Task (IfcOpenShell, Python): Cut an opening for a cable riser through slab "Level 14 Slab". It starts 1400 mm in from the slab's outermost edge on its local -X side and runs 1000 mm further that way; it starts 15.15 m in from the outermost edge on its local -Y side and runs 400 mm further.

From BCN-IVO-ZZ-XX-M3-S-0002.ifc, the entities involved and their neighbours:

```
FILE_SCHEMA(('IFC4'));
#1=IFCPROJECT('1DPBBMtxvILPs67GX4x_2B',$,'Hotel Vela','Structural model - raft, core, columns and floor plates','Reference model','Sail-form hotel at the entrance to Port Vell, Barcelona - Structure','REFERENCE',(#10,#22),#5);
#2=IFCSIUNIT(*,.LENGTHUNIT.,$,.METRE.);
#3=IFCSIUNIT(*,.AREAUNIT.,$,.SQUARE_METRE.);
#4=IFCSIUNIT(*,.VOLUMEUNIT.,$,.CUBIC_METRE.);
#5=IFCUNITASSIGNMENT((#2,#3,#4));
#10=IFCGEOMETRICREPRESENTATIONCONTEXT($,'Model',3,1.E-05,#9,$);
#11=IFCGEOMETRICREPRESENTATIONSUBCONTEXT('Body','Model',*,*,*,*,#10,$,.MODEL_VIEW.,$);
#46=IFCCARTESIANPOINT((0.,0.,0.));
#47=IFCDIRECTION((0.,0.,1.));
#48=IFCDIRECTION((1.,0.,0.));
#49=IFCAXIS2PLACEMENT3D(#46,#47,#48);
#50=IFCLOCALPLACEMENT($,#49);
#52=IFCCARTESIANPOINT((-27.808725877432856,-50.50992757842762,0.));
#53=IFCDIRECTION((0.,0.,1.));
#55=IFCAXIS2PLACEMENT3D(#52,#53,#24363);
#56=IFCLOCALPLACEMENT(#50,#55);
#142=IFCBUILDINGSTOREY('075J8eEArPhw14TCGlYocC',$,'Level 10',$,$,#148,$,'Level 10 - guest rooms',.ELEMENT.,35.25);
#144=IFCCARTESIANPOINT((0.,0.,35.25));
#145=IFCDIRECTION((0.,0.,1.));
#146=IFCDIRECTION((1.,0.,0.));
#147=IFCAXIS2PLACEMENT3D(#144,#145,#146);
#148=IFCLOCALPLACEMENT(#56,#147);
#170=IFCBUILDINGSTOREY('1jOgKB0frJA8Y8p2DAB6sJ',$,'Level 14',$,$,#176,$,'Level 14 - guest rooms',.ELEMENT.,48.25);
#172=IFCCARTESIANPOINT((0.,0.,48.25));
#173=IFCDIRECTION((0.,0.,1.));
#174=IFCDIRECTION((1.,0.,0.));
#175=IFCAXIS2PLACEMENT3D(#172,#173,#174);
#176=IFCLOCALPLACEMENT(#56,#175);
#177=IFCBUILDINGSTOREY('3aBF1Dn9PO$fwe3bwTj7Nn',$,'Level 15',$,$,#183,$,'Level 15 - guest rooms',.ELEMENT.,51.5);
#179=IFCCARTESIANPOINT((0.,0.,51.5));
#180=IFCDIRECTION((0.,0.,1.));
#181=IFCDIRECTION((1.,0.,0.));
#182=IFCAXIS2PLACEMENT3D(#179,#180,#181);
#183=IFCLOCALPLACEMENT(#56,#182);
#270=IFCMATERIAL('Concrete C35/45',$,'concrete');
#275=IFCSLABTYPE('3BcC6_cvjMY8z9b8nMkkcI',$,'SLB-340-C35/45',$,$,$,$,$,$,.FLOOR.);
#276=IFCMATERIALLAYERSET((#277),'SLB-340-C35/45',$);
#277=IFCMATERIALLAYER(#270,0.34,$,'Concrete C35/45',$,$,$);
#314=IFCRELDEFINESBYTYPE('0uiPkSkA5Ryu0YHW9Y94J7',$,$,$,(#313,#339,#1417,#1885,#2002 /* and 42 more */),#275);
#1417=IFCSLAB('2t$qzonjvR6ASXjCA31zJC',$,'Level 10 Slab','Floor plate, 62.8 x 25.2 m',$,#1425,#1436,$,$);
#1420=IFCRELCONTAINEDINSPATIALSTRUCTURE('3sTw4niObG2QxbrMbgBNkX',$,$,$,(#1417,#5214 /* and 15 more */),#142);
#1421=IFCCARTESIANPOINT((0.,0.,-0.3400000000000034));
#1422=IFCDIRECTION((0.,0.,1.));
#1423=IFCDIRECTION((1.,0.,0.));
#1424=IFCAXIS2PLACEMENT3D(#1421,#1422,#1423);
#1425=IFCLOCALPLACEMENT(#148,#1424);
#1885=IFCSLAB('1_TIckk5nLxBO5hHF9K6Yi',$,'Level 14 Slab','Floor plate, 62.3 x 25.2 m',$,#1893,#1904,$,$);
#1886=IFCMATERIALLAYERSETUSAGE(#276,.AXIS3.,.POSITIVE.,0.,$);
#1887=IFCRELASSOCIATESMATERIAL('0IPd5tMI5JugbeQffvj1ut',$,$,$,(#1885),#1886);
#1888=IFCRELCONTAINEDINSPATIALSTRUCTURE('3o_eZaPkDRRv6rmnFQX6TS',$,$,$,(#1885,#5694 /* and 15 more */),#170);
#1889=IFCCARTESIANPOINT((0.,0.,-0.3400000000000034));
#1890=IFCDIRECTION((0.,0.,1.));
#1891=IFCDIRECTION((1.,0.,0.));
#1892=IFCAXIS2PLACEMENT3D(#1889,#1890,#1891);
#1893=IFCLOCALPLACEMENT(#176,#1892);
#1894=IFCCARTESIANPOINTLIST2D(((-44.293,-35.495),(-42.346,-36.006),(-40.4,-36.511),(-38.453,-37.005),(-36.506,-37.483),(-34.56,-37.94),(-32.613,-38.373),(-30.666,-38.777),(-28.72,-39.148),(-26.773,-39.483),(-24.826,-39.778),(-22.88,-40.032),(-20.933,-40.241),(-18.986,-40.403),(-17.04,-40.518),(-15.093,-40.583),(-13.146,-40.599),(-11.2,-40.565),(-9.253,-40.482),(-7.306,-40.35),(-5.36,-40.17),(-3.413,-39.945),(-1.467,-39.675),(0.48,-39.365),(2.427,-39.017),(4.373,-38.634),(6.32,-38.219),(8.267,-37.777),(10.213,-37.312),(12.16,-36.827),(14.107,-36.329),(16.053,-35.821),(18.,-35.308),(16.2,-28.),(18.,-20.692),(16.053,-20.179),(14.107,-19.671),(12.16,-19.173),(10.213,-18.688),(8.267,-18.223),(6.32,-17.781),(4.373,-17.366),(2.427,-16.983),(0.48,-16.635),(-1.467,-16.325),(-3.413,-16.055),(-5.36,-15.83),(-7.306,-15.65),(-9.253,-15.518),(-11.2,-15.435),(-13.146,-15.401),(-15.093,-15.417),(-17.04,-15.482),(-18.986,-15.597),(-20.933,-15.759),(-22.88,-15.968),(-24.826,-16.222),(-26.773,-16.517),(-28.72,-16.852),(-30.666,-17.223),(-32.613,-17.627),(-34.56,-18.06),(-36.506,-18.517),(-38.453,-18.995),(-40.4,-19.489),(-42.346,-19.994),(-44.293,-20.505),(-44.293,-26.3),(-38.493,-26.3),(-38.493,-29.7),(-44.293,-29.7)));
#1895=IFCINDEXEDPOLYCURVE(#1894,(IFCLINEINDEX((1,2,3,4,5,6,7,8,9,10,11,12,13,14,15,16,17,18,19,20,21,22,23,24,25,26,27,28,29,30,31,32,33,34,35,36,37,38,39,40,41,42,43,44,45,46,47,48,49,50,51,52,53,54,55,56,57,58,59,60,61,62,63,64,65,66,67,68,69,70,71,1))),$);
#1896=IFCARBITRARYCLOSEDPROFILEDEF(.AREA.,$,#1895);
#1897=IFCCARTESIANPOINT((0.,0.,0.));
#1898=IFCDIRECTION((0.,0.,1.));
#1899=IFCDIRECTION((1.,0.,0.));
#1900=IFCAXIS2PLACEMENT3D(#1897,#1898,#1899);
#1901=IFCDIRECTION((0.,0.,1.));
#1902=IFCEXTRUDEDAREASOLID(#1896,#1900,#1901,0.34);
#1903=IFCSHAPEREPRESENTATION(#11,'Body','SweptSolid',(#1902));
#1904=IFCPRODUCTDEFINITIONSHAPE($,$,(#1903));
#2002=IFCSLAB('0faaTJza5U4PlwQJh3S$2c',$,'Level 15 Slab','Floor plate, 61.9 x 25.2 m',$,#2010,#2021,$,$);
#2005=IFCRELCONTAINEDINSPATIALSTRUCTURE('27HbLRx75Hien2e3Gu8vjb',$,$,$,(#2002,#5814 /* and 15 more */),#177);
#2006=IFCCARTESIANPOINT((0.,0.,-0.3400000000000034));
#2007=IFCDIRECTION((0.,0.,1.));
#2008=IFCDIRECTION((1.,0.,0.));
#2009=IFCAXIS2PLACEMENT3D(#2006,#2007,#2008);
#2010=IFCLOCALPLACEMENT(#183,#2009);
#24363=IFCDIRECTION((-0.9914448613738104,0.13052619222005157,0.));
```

```python
import numpy as np
import ifcopenshell
import ifcopenshell.api.feature
import ifcopenshell.api.geometry
import ifcopenshell.api.root
import ifcopenshell.geom
import ifcopenshell.util.placement
import ifcopenshell.util.representation
import ifcopenshell.util.shape
import ifcopenshell.util.unit

model = ifcopenshell.open("BCN-IVO-ZZ-XX-M3-S-0002.ifc")
unit_scale = ifcopenshell.util.unit.calculate_unit_scale(model)
settings = ifcopenshell.geom.settings()


def volume(element):
    """Net volume in cubic metres, openings subtracted."""
    shape = ifcopenshell.geom.create_shape(settings, element)
    return ifcopenshell.util.shape.get_volume(shape.geometry)


slab = model.by_id(1885)
before = volume(slab)

# Extent in the slab's own axes, in metres. The edges named are its -X and -Y sides.
slab_shape = ifcopenshell.geom.create_shape(settings, slab)
vertices = ifcopenshell.util.shape.get_vertices(slab_shape.geometry)
x_min, y_min, bottom = vertices.min(axis=0)
top = vertices[:, 2].max()

opening = ifcopenshell.api.root.create_entity(model, ifc_class="IfcOpeningElement", name="Cable riser opening", predefined_type="OPENING")
context = ifcopenshell.util.representation.get_context(model, "Model", "Body", "MODEL_VIEW")
width, depth = 1, 0.4
outline = [(0.0, 0.0), (width, 0.0), (width, depth), (0.0, depth), (0.0, 0.0)]
# Overshoot both faces by 50 mm so the cut is clean.
shape = ifcopenshell.api.geometry.add_slab_representation(
    model, context=context, depth=top - bottom + 0.1, polyline=outline
)
ifcopenshell.api.geometry.assign_representation(model, product=opening, representation=shape)

matrix = ifcopenshell.util.placement.get_local_placement(slab.ObjectPlacement)
matrix[:, 3] = matrix @ np.append(np.array([x_min + 1.4, y_min + 15.15, bottom - 0.05]) / unit_scale, 1.0)
ifcopenshell.api.geometry.edit_object_placement(model, product=opening, matrix=matrix, is_si=False)
ifcopenshell.api.feature.add_feature(model, feature=opening, element=slab)

after = volume(slab)

print(f"slab volume {before:.3f} -> {after:.3f} m3")

model.write("BCN-IVO-ZZ-XX-M3-S-0002_updated.ifc")
```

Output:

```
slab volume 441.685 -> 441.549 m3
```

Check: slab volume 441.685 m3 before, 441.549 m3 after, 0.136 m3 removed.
